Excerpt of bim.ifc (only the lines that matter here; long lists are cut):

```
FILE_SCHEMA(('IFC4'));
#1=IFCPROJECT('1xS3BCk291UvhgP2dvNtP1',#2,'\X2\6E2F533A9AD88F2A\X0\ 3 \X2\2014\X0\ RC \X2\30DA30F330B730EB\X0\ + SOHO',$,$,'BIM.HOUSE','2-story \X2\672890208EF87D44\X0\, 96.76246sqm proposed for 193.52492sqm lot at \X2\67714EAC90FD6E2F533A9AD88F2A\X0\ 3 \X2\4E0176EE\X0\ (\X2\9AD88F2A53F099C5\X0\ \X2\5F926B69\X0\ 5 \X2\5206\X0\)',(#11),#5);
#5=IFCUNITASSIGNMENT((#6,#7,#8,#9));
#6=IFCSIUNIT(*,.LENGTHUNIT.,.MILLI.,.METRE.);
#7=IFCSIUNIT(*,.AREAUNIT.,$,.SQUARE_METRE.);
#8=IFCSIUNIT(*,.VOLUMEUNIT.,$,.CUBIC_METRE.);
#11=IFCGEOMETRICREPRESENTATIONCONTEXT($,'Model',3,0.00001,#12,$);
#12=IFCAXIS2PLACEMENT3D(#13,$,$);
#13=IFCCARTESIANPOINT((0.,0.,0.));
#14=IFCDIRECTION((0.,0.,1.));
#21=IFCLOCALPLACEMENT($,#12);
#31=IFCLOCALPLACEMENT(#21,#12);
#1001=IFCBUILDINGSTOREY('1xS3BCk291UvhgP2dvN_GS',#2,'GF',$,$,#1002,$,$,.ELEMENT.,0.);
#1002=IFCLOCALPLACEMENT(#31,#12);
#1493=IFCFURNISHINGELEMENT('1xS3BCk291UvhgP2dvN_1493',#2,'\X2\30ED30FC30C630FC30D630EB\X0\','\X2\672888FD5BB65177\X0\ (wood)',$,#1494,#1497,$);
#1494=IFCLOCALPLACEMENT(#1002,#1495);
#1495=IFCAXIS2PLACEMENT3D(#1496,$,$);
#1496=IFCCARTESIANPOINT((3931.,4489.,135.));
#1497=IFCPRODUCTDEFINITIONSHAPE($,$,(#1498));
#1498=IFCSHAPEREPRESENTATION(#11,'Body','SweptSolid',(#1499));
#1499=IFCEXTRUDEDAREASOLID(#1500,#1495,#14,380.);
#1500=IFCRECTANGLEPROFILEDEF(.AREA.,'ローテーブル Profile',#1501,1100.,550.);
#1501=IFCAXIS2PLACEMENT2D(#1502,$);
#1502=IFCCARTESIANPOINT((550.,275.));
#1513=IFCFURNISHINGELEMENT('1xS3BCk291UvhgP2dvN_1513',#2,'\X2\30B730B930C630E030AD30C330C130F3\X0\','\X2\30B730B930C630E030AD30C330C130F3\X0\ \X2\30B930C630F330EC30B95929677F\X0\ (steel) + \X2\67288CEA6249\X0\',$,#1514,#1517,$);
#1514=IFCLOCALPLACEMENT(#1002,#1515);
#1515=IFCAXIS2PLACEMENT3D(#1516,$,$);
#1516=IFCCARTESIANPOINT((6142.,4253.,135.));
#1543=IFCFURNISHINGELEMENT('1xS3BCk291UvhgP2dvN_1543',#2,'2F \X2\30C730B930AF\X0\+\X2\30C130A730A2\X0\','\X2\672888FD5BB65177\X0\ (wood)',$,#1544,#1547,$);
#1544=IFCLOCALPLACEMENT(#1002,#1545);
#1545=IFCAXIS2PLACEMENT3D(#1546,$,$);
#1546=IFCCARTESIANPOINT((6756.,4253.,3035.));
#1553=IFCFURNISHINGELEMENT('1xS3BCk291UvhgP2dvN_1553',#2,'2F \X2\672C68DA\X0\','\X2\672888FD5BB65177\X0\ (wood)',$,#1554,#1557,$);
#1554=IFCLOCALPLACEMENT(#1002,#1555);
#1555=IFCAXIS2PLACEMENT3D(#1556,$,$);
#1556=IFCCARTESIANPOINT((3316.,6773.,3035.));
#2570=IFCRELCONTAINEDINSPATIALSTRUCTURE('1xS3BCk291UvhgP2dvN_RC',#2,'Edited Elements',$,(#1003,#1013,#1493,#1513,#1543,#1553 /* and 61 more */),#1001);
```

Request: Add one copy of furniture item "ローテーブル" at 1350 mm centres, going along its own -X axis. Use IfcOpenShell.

```python
import ifcopenshell
import ifcopenshell.api.geometry
import ifcopenshell.api.root
import ifcopenshell.util.element
import ifcopenshell.util.placement
import ifcopenshell.util.unit

model = ifcopenshell.open("bim.ifc")
unit_scale = ifcopenshell.util.unit.calculate_unit_scale(model)


def reuse_history(source, copy):
    """copy_class also copies each property set's owner history, people and application; keep the originals."""
    for rel in copy.IsDefinedBy:
        if rel.is_a("IfcRelDefinesByProperties") and (history := rel.RelatingPropertyDefinition.OwnerHistory):
            rel.RelatingPropertyDefinition.OwnerHistory = source.OwnerHistory
            ifcopenshell.util.element.remove_deep2(model, history)


source = model.by_id(1493)
base = ifcopenshell.util.placement.get_local_placement(source.ObjectPlacement)
step = -base[:3, 0] * 1.35 / unit_scale

for i in range(1, 2):
    copy = ifcopenshell.api.root.copy_class(model, product=source)
    copy.Representation = ifcopenshell.util.element.copy_deep(
        model, source.Representation, exclude=["IfcGeometricRepresentationContext", "IfcRepresentationMap"]
    )
    reuse_history(source, copy)
    matrix = base.copy()
    matrix[:3, 3] += i * step
    print("added at", matrix[:3, 3].round(3) + 0.0)
    ifcopenshell.api.geometry.edit_object_placement(model, product=copy, matrix=matrix, is_si=False)

model.write("bim_rev.ifc")
```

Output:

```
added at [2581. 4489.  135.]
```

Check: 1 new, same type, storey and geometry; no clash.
